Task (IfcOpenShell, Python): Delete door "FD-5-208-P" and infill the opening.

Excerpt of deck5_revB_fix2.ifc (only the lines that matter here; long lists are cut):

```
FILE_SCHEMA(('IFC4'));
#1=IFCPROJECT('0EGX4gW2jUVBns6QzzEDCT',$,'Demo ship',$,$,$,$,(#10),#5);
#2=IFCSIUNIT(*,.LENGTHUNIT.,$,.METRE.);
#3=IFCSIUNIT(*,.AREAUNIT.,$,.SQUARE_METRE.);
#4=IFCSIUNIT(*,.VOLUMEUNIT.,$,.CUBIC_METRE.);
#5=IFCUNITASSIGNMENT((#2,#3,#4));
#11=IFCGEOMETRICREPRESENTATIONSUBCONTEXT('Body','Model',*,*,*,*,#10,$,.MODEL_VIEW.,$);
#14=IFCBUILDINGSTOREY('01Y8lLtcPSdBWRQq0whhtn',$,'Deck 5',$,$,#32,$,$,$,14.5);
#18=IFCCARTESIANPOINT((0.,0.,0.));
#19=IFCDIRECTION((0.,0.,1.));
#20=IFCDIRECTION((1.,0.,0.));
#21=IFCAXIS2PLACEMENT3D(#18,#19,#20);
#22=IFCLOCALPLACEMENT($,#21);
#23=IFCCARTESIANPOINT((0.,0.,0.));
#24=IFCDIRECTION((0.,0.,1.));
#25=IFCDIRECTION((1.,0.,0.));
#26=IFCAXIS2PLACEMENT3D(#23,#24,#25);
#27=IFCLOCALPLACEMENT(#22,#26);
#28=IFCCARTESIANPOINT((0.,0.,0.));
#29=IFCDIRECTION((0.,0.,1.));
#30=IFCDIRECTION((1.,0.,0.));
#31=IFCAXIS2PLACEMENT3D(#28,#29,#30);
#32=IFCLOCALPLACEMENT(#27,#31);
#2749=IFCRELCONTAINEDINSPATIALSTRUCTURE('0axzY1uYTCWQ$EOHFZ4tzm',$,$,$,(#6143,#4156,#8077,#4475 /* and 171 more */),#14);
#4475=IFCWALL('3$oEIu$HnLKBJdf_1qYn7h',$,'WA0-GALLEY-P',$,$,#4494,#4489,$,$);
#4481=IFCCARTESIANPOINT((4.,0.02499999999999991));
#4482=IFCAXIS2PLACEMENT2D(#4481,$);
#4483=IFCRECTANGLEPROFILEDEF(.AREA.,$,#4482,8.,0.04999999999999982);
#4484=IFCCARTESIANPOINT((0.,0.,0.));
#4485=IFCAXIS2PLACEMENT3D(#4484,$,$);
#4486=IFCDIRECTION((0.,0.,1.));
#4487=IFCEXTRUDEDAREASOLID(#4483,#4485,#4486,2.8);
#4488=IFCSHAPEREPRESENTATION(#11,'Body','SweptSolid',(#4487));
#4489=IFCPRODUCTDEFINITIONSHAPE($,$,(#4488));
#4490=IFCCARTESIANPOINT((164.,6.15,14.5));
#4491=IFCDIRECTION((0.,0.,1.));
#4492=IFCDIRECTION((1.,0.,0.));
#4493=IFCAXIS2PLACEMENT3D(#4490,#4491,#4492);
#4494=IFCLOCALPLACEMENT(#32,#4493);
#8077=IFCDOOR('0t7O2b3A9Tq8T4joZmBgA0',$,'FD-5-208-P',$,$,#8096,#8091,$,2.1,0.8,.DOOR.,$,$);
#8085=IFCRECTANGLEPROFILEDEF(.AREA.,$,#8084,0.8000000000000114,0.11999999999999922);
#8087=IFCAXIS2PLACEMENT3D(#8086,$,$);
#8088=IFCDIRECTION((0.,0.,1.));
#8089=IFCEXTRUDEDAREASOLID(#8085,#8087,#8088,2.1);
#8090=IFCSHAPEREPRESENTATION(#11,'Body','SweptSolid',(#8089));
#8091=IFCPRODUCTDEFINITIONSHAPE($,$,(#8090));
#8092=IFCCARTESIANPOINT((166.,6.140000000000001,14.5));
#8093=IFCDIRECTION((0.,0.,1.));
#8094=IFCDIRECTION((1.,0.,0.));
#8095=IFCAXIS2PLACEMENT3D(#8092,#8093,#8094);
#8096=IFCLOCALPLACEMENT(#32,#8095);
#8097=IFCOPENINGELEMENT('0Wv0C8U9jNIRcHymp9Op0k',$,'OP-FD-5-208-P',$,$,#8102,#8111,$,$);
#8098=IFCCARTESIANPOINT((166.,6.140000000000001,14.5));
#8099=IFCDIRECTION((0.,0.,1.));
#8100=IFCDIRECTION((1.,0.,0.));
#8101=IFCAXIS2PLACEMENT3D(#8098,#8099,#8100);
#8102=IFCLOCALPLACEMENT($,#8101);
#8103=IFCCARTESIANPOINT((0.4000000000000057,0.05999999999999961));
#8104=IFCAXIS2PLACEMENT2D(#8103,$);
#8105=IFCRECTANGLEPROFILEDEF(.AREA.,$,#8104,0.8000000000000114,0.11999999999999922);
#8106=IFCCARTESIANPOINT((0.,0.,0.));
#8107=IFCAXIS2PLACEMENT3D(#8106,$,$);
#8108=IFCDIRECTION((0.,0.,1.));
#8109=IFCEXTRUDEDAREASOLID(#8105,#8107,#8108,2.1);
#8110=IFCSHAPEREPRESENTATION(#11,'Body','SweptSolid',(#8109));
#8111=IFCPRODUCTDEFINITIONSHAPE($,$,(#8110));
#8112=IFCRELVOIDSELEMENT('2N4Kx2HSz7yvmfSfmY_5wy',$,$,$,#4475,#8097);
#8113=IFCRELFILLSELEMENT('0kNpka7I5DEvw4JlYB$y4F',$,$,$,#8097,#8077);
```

```python
import ifcopenshell
import ifcopenshell.api.feature
import ifcopenshell.api.root
import ifcopenshell.geom
import ifcopenshell.util.shape

model = ifcopenshell.open("deck5_revB_fix2.ifc")
settings = ifcopenshell.geom.settings()


def volume(element):
    """Net volume in cubic metres, openings subtracted."""
    shape = ifcopenshell.geom.create_shape(settings, element)
    return ifcopenshell.util.shape.get_volume(shape.geometry)


door = model.by_guid("0t7O2b3A9Tq8T4joZmBgA0")
opening = door.FillsVoids[0].RelatingOpeningElement
wall = opening.VoidsElements[0].RelatingBuildingElement
before = volume(wall)

ifcopenshell.api.root.remove_product(model, product=door)
ifcopenshell.api.feature.remove_feature(model, feature=opening)

after = volume(wall)

print(f"wall volume {before:.3f} -> {after:.3f} m3")

model.write("deck5_revB_fix2_edited.ifc")
```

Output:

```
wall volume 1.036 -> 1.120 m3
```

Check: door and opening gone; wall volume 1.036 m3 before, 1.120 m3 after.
